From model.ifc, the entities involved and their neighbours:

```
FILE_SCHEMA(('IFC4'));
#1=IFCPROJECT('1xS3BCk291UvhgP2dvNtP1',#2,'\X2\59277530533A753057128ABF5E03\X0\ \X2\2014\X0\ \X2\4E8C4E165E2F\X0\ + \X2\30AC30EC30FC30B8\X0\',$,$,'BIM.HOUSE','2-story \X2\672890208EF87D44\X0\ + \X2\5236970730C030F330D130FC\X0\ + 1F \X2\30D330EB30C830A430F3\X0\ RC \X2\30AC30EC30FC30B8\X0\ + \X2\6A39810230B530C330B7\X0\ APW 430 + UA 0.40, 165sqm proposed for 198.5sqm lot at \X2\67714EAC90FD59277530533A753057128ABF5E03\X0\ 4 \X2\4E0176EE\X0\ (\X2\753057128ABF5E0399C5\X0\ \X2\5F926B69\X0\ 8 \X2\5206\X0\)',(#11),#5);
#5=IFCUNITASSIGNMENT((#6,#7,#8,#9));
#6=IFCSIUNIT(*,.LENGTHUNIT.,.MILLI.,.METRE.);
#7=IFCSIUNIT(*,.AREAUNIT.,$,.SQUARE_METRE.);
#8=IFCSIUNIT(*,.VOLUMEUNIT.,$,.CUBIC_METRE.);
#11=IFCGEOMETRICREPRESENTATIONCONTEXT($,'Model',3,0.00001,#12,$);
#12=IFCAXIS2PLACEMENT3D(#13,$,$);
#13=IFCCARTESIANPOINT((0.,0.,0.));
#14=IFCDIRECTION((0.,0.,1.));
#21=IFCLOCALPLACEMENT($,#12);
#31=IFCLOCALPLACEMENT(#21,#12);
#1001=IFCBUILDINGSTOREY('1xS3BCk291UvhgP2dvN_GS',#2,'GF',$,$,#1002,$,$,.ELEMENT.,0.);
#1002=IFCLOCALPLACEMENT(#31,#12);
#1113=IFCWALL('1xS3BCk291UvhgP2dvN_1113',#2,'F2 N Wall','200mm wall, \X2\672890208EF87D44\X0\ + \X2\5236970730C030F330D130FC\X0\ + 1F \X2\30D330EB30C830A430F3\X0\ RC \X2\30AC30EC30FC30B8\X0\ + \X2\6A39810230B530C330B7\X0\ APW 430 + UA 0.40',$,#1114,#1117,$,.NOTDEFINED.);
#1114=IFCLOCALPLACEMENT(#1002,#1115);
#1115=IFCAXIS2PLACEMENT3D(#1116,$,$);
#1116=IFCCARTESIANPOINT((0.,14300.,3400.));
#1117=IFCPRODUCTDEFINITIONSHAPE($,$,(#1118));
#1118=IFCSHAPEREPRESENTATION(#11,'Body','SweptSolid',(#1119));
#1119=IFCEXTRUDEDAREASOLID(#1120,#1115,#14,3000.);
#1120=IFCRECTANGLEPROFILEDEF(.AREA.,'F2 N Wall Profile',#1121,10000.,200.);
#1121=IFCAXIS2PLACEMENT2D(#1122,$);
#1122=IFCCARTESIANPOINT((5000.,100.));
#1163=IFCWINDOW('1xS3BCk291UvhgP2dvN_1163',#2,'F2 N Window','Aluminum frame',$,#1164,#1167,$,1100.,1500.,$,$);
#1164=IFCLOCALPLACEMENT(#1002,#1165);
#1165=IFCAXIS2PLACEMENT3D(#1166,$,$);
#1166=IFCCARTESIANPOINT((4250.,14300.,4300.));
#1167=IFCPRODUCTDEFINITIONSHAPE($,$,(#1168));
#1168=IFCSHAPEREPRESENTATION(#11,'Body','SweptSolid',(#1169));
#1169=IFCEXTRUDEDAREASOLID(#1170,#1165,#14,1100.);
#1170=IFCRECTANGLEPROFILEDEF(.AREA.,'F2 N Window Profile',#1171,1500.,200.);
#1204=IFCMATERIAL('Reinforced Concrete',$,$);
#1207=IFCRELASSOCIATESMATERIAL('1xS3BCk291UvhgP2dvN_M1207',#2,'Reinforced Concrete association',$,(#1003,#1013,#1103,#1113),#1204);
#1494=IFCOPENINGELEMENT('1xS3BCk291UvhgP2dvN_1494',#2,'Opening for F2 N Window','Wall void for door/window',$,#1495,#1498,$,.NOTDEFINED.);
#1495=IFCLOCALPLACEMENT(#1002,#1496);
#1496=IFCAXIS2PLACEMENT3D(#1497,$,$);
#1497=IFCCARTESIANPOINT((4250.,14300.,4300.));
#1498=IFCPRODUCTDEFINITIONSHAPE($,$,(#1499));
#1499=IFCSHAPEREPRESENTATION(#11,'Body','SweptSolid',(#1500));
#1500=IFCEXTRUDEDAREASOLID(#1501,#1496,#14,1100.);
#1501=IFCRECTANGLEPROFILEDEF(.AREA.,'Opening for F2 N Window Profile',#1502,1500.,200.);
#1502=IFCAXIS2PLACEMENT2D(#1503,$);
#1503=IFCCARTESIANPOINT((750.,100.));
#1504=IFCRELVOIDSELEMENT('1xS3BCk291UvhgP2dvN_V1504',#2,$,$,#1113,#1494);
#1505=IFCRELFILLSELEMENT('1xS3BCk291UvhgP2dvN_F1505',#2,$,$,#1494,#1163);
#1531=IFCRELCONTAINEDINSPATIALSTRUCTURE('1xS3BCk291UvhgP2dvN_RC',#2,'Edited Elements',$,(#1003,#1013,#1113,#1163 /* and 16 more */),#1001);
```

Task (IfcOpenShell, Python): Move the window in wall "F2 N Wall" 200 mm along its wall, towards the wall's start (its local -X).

```python
import ifcopenshell
import ifcopenshell.api.geometry
import ifcopenshell.util.placement
import ifcopenshell.util.unit

model = ifcopenshell.open("model.ifc")
unit_scale = ifcopenshell.util.unit.calculate_unit_scale(model)

window = model.by_id(1163)
opening = window.FillsVoids[0].RelatingOpeningElement
wall = opening.VoidsElements[0].RelatingBuildingElement

wall_matrix = ifcopenshell.util.placement.get_local_placement(wall.ObjectPlacement)
shift = wall_matrix[:3, 0] * -0.2 / unit_scale
before = ifcopenshell.util.placement.get_local_placement(window.ObjectPlacement)[:3, 3].copy()

# The window is not placed relative to its opening, so move both.
for product in (opening, window):
    matrix = ifcopenshell.util.placement.get_local_placement(product.ObjectPlacement)
    matrix[:3, 3] += shift
    ifcopenshell.api.geometry.edit_object_placement(model, product=product, matrix=matrix, is_si=False)

after = ifcopenshell.util.placement.get_local_placement(window.ObjectPlacement)[:3, 3]
print("window moved by", (after - before).round(3) + 0.0)

model.write("model_v2.ifc")
```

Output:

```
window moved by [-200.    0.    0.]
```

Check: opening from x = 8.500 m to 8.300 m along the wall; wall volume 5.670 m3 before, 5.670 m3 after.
